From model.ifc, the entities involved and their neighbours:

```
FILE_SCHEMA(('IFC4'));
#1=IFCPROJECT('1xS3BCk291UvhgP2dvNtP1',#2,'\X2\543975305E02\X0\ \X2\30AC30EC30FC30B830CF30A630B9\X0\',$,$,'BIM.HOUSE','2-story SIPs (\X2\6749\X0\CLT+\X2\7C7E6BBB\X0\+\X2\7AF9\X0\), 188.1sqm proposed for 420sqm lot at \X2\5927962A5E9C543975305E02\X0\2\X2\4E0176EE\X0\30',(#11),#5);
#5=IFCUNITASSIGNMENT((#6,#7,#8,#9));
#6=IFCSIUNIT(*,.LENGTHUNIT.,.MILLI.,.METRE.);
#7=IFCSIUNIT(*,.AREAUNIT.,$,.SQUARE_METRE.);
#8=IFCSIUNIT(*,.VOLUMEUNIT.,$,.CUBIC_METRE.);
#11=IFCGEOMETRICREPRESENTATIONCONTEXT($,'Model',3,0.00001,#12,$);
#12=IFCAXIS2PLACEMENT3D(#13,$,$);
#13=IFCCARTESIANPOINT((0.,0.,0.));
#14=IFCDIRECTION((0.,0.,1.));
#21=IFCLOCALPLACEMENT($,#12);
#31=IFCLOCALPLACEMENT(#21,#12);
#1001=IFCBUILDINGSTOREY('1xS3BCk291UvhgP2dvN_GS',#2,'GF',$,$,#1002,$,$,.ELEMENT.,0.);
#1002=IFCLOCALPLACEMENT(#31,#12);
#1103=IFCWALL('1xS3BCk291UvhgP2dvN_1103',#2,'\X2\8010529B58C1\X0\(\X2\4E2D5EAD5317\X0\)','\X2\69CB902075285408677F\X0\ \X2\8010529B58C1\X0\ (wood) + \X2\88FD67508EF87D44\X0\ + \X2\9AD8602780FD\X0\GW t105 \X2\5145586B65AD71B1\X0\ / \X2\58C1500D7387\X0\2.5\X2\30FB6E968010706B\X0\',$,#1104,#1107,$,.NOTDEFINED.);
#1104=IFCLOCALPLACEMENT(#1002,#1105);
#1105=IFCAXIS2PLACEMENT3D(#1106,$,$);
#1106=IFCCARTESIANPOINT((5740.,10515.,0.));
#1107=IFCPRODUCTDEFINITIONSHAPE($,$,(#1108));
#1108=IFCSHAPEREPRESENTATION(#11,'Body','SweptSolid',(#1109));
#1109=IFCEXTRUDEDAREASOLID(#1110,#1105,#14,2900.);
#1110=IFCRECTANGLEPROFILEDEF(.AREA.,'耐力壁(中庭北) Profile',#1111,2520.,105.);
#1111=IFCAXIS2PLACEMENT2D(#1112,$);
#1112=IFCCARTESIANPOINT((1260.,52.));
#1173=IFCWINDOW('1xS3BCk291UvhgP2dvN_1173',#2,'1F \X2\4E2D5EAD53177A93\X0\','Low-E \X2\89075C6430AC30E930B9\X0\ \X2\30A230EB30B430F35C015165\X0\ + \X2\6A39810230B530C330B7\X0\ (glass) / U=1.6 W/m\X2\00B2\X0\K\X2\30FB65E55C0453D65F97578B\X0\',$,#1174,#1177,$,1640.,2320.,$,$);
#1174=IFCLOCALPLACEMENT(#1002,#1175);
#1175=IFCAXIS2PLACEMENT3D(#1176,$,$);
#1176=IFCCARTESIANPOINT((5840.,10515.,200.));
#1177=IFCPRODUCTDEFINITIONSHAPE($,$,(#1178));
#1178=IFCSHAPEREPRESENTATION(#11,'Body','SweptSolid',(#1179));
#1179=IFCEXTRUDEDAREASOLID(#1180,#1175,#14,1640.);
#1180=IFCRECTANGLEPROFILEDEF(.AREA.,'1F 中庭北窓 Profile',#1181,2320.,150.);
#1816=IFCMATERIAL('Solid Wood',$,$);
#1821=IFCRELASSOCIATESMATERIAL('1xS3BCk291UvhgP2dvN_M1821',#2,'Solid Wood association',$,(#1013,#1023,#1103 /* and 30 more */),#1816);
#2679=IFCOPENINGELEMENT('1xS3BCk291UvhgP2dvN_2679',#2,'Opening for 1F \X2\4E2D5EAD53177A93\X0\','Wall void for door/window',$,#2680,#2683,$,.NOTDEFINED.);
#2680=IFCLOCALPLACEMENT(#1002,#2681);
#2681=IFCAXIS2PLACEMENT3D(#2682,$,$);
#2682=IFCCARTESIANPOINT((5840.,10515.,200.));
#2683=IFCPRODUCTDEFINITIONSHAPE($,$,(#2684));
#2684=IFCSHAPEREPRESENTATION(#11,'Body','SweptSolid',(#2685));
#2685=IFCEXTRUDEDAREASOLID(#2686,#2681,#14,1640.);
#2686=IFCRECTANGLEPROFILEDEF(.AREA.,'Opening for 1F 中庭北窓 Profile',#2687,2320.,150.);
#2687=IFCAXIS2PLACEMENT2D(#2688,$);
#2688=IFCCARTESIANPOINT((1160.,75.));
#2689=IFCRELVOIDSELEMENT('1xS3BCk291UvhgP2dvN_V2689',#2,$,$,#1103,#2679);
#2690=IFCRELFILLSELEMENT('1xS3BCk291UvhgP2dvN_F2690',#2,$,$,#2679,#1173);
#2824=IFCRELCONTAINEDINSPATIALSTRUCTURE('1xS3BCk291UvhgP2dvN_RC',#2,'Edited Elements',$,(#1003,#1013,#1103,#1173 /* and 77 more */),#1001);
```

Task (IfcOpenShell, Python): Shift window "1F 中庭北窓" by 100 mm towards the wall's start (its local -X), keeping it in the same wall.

```python
import ifcopenshell
import ifcopenshell.api.geometry
import ifcopenshell.util.placement
import ifcopenshell.util.unit

model = ifcopenshell.open("model.ifc")
unit_scale = ifcopenshell.util.unit.calculate_unit_scale(model)

window = model.by_guid("1xS3BCk291UvhgP2dvN_1173")
opening = window.FillsVoids[0].RelatingOpeningElement
wall = opening.VoidsElements[0].RelatingBuildingElement

wall_matrix = ifcopenshell.util.placement.get_local_placement(wall.ObjectPlacement)
shift = wall_matrix[:3, 0] * -0.1 / unit_scale
before = ifcopenshell.util.placement.get_local_placement(window.ObjectPlacement)[:3, 3].copy()

# The window is not placed relative to its opening, so move both.
for product in (opening, window):
    matrix = ifcopenshell.util.placement.get_local_placement(product.ObjectPlacement)
    matrix[:3, 3] += shift
    ifcopenshell.api.geometry.edit_object_placement(model, product=product, matrix=matrix, is_si=False)

after = ifcopenshell.util.placement.get_local_placement(window.ObjectPlacement)[:3, 3]
print("window moved by", (after - before).round(3) + 0.0)

model.write("model_updated.ifc")
```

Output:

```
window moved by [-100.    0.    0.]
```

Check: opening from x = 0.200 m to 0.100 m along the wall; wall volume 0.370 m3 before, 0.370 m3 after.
